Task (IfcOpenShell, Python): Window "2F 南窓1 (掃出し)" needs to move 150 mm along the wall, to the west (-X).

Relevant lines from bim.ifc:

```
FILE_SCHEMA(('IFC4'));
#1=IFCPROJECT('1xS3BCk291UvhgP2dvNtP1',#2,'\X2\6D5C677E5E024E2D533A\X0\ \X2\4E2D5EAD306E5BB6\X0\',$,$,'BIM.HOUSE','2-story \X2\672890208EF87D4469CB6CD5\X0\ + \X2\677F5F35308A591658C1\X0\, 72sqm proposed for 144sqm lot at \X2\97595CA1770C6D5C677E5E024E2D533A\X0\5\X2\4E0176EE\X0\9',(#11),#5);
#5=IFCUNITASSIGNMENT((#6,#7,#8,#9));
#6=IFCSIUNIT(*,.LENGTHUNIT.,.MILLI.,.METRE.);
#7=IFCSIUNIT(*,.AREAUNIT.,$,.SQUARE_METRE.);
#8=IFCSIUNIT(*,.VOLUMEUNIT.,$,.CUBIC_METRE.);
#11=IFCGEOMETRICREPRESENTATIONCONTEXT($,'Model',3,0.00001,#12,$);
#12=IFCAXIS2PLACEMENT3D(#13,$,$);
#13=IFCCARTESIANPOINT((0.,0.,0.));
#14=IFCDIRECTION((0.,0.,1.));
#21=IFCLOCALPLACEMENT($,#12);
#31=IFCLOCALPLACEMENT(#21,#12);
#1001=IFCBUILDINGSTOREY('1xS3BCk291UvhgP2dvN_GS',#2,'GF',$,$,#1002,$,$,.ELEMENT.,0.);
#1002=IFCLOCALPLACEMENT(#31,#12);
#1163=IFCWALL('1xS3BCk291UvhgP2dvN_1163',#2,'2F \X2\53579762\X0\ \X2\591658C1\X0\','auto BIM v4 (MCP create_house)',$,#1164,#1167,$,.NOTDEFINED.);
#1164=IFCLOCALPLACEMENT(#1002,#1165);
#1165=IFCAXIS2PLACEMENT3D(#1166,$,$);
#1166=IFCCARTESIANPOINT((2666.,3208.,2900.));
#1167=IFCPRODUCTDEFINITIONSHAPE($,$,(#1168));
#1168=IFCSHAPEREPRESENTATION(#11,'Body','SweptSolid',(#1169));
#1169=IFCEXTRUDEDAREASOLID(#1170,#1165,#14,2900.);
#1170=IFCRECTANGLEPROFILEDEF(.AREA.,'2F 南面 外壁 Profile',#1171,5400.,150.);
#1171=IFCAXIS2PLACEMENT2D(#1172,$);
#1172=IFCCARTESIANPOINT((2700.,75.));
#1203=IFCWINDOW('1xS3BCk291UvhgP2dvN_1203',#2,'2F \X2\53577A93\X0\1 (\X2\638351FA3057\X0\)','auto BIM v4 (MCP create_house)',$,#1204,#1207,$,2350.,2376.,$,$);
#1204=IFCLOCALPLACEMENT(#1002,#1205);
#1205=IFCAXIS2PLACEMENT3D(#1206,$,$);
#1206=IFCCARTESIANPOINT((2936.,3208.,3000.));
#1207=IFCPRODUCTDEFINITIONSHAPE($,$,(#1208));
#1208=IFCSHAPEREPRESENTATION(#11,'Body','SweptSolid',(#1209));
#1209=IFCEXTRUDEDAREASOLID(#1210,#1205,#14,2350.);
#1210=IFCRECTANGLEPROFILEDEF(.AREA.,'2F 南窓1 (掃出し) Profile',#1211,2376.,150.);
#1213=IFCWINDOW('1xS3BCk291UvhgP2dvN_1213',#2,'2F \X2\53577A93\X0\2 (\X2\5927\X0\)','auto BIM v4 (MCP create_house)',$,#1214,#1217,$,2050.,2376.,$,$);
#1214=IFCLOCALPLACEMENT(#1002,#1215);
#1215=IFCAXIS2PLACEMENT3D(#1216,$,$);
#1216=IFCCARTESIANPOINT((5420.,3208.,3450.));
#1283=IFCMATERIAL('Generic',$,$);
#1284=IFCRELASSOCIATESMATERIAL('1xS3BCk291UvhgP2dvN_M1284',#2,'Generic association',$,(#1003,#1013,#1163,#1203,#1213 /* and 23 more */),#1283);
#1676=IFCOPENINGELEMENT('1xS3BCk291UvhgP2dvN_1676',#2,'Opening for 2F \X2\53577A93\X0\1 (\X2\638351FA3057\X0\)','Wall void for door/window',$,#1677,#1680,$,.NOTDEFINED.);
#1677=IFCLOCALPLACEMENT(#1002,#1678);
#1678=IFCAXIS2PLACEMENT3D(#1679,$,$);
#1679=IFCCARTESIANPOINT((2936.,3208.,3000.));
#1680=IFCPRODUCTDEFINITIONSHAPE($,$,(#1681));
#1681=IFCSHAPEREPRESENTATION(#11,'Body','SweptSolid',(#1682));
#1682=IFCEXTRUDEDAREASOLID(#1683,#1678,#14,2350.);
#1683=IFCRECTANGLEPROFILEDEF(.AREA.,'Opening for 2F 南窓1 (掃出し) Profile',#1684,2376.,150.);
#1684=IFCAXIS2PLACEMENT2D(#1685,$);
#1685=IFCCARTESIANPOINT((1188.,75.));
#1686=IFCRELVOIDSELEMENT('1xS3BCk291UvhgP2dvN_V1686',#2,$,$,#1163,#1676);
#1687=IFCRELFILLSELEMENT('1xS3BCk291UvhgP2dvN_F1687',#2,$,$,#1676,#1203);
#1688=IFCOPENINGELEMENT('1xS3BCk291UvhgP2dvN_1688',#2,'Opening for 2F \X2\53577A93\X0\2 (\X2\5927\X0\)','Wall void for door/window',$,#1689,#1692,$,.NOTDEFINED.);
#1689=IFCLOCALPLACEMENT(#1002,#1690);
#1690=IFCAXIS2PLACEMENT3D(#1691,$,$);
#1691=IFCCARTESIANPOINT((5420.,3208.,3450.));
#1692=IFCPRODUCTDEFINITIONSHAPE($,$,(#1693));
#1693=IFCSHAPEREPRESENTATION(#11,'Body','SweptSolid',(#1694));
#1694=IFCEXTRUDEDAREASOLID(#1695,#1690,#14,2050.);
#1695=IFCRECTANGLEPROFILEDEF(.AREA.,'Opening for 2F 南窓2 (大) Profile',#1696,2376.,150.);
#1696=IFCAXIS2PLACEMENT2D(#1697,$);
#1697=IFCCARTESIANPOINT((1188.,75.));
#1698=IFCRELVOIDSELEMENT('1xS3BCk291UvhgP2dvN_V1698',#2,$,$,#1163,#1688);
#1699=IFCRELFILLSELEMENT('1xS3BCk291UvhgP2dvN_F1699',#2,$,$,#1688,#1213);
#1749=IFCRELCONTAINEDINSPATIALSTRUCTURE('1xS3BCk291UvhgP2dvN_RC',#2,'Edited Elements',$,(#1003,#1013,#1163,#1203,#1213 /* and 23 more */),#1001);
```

```python
import ifcopenshell
import ifcopenshell.api.geometry
import ifcopenshell.util.placement

model = ifcopenshell.open("bim.ifc")

window = model.by_guid("1xS3BCk291UvhgP2dvN_1203")
opening = window.FillsVoids[0].RelatingOpeningElement
wall = opening.VoidsElements[0].RelatingBuildingElement

wall_matrix = ifcopenshell.util.placement.get_local_placement(wall.ObjectPlacement)
shift = wall_matrix[:3, 0] * -150.0
before = ifcopenshell.util.placement.get_local_placement(window.ObjectPlacement)[:3, 3].copy()

# The window is not placed relative to its opening, so move both.
for product in (opening, window):
    matrix = ifcopenshell.util.placement.get_local_placement(product.ObjectPlacement)
    matrix[:3, 3] += shift
    ifcopenshell.api.geometry.edit_object_placement(model, product=product, matrix=matrix, is_si=False)

after = ifcopenshell.util.placement.get_local_placement(window.ObjectPlacement)[:3, 3]
print("window moved by", (after - before).round(3) + 0.0)

model.write("bim_edited.ifc")
```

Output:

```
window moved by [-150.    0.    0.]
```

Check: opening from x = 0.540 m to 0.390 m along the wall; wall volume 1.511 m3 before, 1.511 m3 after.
